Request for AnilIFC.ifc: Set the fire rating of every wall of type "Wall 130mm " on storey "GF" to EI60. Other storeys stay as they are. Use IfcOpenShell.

First a look at what the model holds.

```python
import ifcopenshell
import ifcopenshell.util.element

model = ifcopenshell.open("AnilIFC.ifc")
print(model.schema)
storey = next(s for s in model.by_type("IfcBuildingStorey") if s.Name == "GF")
walls = [e for e in ifcopenshell.util.element.get_decomposition(storey) if e.is_a("IfcWall")]
seen = {}
for e in walls:
    element_type = ifcopenshell.util.element.get_type(e)
    key = (element_type.Name if element_type != e and element_type else None, ifcopenshell.util.element.get_pset(e, "Pset_WallCommon", "FireRating"))
    seen[key] = seen.get(key, 0) + 1
for (name, value), count in sorted(seen.items(), key=str):
    print(count, "x", name, "|", value)
```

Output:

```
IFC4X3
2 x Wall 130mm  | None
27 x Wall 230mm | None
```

```python
import ifcopenshell
import ifcopenshell.api.pset
import ifcopenshell.util.element

model = ifcopenshell.open("AnilIFC.ifc")

storey = next(s for s in model.by_type("IfcBuildingStorey") if s.Name == "GF")
walls = [e for e in ifcopenshell.util.element.get_decomposition(storey) if e.is_a("IfcWall")]

count = 0
for e in walls:
    element_type = ifcopenshell.util.element.get_type(e)
    if element_type in (None, e) or element_type.Name != "Wall 130mm ":
        continue
    # add_pset returns the element's existing set when there is one.
    pset = ifcopenshell.api.pset.add_pset(model, product=e, name="Pset_WallCommon")
    ifcopenshell.api.pset.edit_pset(model, pset=pset, properties={"FireRating": "EI60"})
    count += 1

print(count, "walls updated")

model.write("AnilIFC_updated.ifc")
```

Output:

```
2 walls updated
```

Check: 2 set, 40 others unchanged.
